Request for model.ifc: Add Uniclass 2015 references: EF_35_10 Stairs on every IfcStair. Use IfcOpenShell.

First a look at what the model holds.

```python
import ifcopenshell

model = ifcopenshell.open("model.ifc")
print(model.schema)
print("classifications:", [c.Name for c in model.by_type("IfcClassification")])
for ifc_class in ("IfcDoor", "IfcRoof", "IfcStair", "IfcWall", "IfcWindow"):
    print(ifc_class, len(model.by_type(ifc_class)))
```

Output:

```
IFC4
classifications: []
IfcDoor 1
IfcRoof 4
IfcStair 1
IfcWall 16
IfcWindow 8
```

```python
import ifcopenshell
import ifcopenshell.api.classification

model = ifcopenshell.open("model.ifc")

system = ifcopenshell.api.classification.add_classification(model, classification="Uniclass 2015")

codes = {
    "IfcStair": ("EF_35_10", "Stairs"),
}
for ifc_class, (code, name) in codes.items():
    products = model.by_type(ifc_class)
    ifcopenshell.api.classification.add_reference(
        model, products=products, classification=system, identification=code, name=name
    )
    print(code, len(products))

model.write("model_rev.ifc")
```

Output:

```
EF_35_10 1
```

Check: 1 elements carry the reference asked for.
